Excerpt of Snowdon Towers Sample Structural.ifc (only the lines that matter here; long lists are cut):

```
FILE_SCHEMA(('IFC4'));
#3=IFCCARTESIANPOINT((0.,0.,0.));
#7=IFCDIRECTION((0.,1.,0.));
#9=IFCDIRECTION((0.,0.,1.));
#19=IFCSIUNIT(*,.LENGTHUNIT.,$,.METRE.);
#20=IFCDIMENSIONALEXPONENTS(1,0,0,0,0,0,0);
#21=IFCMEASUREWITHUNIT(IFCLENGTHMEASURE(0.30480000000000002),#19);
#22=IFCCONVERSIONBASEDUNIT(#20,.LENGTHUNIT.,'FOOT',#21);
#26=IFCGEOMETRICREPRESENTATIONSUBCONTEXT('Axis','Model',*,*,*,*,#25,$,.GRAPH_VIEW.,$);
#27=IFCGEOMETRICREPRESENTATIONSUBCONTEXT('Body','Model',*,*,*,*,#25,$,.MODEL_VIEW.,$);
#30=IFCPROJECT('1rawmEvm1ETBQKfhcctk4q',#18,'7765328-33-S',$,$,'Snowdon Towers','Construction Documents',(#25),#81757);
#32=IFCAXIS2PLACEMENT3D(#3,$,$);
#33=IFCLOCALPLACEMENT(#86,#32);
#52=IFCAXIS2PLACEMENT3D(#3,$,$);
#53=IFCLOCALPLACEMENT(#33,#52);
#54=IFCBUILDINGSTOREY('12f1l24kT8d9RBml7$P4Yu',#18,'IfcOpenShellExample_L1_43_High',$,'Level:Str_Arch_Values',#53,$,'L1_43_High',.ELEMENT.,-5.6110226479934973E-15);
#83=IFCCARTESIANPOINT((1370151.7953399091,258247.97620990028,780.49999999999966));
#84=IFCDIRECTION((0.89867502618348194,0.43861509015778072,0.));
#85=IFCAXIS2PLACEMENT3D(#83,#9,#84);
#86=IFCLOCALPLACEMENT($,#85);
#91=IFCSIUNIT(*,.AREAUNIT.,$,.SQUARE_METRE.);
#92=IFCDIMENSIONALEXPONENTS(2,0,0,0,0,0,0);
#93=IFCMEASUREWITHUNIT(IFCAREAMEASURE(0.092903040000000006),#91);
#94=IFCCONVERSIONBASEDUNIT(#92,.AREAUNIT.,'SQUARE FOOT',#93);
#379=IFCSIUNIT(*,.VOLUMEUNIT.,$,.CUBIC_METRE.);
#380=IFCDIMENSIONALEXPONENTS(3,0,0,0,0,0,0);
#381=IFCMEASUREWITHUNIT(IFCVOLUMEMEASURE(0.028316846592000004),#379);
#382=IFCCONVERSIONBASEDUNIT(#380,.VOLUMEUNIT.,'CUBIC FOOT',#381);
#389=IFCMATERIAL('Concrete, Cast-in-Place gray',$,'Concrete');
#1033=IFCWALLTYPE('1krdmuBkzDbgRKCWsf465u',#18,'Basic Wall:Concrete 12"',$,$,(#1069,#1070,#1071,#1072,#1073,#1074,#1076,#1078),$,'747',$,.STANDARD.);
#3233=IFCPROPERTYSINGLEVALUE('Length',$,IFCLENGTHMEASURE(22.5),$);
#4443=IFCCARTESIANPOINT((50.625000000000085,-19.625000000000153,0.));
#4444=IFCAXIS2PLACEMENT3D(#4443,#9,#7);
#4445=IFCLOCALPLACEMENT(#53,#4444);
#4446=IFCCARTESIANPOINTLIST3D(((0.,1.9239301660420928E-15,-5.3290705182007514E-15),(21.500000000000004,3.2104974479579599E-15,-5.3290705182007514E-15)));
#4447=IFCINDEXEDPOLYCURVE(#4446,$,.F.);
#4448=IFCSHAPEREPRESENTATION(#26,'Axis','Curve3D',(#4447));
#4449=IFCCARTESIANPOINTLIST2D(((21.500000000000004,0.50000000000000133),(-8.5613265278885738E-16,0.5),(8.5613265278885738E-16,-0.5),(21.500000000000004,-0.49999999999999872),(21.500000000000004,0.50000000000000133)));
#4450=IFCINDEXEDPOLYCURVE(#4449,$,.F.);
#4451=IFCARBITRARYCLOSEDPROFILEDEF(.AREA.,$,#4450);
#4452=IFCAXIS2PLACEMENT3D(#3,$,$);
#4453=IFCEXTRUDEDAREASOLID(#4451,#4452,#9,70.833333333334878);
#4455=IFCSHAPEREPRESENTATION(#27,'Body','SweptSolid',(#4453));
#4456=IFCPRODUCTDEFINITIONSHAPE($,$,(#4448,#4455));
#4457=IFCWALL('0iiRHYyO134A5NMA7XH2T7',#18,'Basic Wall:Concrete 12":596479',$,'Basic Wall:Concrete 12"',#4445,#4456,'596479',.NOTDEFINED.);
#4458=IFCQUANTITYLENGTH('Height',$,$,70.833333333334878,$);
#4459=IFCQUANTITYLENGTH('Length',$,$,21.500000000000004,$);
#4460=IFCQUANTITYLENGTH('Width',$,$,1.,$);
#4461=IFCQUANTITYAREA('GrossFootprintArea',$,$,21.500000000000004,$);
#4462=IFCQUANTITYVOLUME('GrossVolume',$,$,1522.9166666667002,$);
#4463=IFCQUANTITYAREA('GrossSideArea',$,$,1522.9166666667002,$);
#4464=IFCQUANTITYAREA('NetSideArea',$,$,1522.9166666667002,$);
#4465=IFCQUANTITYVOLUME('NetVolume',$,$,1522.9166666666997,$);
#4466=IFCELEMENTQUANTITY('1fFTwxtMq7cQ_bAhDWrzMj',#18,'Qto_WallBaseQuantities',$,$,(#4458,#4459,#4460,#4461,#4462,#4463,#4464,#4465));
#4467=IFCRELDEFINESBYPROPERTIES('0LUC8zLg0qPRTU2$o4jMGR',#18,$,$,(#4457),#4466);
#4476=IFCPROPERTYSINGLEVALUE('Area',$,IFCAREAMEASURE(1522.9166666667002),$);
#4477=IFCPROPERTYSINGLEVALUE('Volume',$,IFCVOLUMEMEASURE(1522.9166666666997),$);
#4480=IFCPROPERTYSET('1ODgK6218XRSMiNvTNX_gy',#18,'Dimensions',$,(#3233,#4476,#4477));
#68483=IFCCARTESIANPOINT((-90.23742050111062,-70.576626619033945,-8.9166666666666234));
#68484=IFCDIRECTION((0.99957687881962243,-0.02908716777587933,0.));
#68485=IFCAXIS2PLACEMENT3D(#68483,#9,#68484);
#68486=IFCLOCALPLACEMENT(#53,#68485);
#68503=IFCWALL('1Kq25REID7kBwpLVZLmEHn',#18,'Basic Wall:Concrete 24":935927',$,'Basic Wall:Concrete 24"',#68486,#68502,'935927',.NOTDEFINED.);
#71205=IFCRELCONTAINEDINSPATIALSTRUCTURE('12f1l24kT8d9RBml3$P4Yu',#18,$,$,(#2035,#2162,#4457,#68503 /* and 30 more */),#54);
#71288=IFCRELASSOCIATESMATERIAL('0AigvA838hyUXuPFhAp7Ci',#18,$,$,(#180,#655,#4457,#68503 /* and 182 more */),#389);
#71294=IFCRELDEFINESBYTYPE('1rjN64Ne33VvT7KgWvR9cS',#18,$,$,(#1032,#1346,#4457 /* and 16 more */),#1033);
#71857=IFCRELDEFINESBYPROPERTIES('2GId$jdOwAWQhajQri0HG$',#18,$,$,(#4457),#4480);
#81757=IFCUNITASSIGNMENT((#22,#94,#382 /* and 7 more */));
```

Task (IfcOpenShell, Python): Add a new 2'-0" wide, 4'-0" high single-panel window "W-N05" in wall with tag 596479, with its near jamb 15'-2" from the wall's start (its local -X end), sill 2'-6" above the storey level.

```python
import numpy as np
import ifcopenshell
import ifcopenshell.api.feature
import ifcopenshell.api.geometry
import ifcopenshell.api.pset
import ifcopenshell.api.root
import ifcopenshell.api.spatial
import ifcopenshell.geom
import ifcopenshell.util.element
import ifcopenshell.util.placement
import ifcopenshell.util.representation
import ifcopenshell.util.shape
import ifcopenshell.util.unit

model = ifcopenshell.open("Snowdon Towers Sample Structural.ifc")
unit_scale = ifcopenshell.util.unit.calculate_unit_scale(model)
area_scale = ifcopenshell.util.unit.calculate_unit_scale(model, "AREAUNIT")
volume_scale = ifcopenshell.util.unit.calculate_unit_scale(model, "VOLUMEUNIT")
settings = ifcopenshell.geom.settings()


def volume(element):
    """Net volume in cubic metres, openings subtracted."""
    shape = ifcopenshell.geom.create_shape(settings, element)
    return ifcopenshell.util.shape.get_volume(shape.geometry)


wall = model.by_guid("0iiRHYyO134A5NMA7XH2T7")
storey = ifcopenshell.util.element.get_container(wall, ifc_class="IfcBuildingStorey")
context = ifcopenshell.util.representation.get_context(model, "Model", "Body", "MODEL_VIEW")
before = volume(wall)

width, height, from_end, sill = 0.6096, 1.2192, 4.6228, 0.762  # metres

# The wall runs along its own X axis, and the end named is its -X end.
wall_shape = ifcopenshell.geom.create_shape(settings, wall)
x, y, z = ifcopenshell.util.shape.get_vertices(wall_shape.geometry).T
start = x.min() + from_end
face, thickness = float(y.min()), float(y.max() - y.min())
wall_matrix = ifcopenshell.util.placement.get_local_placement(wall.ObjectPlacement)
level = ifcopenshell.util.placement.get_local_placement(storey.ObjectPlacement)[2, 3]


def in_wall(x, y):
    """Placement at x, y metres in the wall's axes, at sill height."""
    matrix = wall_matrix.copy()
    matrix[:, 3] = wall_matrix @ np.array([x / unit_scale, y / unit_scale, 0.0, 1.0])
    matrix[2, 3] = level + sill / unit_scale
    return matrix


# Opening: a box that overshoots both wall faces by 50 mm.
opening = ifcopenshell.api.root.create_entity(model, ifc_class="IfcOpeningElement", predefined_type="OPENING")
box = ifcopenshell.api.geometry.add_wall_representation(
    model, context=context, length=width, height=height, thickness=thickness + 0.1
)
ifcopenshell.api.geometry.assign_representation(model, product=opening, representation=box)
ifcopenshell.api.geometry.edit_object_placement(model, product=opening, matrix=in_wall(start, face - 0.05), is_si=False)
ifcopenshell.api.feature.add_feature(model, feature=opening, element=wall)

window = ifcopenshell.api.root.create_entity(model, ifc_class="IfcWindow", name="W-N05", predefined_type="WINDOW")
window.OverallWidth, window.OverallHeight = width / unit_scale, height / unit_scale
window.PartitioningType = "SINGLE_PANEL"
body = ifcopenshell.api.geometry.add_window_representation(
    model,
    context=context,
    overall_width=window.OverallWidth,
    overall_height=window.OverallHeight,
    partition_type="SINGLE_PANEL",
)
ifcopenshell.api.geometry.assign_representation(model, product=window, representation=body)
ifcopenshell.api.spatial.assign_container(model, products=[window], relating_structure=storey)
ifcopenshell.api.feature.add_filling(model, opening=opening, element=window)

# Centre the window in the wall's thickness.
ifcopenshell.api.geometry.edit_object_placement(model, product=window, matrix=in_wall(start, face), is_si=False)
window_shape = ifcopenshell.geom.create_shape(settings, window)
depth = ifcopenshell.util.shape.get_vertices(window_shape.geometry)[:, 1]
offset = face + thickness / 2 - (depth.min() + depth.max()) / 2
ifcopenshell.api.geometry.edit_object_placement(model, product=window, matrix=in_wall(start, offset), is_si=False)

after = volume(wall)

# Update the wall's stored quantities.
qto = model.by_id(ifcopenshell.util.element.get_pset(wall, "Qto_WallBaseQuantities", should_inherit=False)["id"])
ifcopenshell.api.pset.edit_qto(model, qto=qto, properties={
    "NetSideArea": after / thickness / area_scale,
    "NetVolume": after / volume_scale,
})
pset = model.by_id(ifcopenshell.util.element.get_pset(wall, "Dimensions", should_inherit=False)["id"])
ifcopenshell.api.pset.edit_pset(model, pset=pset, properties={
    "Area": model.create_entity("IfcAreaMeasure", after / thickness / area_scale),
    "Volume": model.create_entity("IfcVolumeMeasure", after / volume_scale),
})

print(f"wall volume {before:.3f} -> {after:.3f} m3")

model.write("Snowdon Towers Sample Structural_v2.ifc")
```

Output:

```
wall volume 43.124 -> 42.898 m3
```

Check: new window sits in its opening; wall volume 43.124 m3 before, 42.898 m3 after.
